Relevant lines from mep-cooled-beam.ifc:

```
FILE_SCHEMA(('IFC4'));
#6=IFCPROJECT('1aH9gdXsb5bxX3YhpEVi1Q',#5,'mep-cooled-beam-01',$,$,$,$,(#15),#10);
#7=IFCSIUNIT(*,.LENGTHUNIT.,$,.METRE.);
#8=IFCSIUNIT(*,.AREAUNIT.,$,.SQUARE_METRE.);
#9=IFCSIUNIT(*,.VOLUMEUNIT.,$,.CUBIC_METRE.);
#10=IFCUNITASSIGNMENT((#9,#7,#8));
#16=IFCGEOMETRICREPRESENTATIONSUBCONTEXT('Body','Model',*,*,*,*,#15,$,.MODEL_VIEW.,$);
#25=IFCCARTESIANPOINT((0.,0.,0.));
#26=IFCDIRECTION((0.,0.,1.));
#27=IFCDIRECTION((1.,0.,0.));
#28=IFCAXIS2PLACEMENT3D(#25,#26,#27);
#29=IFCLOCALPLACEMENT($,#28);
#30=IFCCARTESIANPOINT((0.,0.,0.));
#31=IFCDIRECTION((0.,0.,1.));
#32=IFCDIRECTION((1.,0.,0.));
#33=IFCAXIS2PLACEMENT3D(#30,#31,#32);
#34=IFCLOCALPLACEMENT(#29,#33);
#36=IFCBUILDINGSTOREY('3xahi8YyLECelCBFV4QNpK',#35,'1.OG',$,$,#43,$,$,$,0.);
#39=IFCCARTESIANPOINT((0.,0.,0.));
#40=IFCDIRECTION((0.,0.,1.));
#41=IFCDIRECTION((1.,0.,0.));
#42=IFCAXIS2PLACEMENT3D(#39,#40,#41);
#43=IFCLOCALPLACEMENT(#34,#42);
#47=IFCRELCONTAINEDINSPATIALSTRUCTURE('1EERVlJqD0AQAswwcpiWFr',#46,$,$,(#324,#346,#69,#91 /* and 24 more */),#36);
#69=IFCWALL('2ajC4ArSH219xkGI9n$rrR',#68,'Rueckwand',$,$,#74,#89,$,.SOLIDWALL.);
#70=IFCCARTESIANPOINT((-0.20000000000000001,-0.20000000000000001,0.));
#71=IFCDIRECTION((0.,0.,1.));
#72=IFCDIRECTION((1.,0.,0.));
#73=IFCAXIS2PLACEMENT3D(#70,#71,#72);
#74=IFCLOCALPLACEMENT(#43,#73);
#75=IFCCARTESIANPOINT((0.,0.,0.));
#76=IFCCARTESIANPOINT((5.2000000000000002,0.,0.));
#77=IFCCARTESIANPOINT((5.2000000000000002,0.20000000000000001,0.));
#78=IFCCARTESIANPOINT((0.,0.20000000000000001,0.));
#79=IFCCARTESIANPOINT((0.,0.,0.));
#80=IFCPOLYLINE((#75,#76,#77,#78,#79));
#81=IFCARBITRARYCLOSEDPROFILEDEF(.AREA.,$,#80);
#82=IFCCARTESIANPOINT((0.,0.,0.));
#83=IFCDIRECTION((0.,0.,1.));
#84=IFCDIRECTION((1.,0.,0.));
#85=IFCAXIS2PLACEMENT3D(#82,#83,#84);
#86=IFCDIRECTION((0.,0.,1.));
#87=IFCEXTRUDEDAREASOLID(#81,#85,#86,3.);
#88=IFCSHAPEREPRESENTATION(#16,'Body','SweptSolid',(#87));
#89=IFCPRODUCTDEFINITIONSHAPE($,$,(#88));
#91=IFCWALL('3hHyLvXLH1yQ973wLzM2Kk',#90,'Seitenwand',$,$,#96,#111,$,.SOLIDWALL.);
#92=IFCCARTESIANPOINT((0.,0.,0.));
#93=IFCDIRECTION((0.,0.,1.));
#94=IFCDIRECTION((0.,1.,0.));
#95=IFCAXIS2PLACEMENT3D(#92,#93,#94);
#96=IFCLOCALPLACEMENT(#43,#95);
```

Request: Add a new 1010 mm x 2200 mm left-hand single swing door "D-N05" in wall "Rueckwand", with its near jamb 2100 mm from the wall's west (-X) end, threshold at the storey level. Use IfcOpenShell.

```python
import numpy as np
import ifcopenshell
import ifcopenshell.api.feature
import ifcopenshell.api.geometry
import ifcopenshell.api.root
import ifcopenshell.api.spatial
import ifcopenshell.geom
import ifcopenshell.util.element
import ifcopenshell.util.placement
import ifcopenshell.util.representation
import ifcopenshell.util.shape
import ifcopenshell.util.unit

model = ifcopenshell.open("mep-cooled-beam.ifc")
unit_scale = ifcopenshell.util.unit.calculate_unit_scale(model)
settings = ifcopenshell.geom.settings()


def volume(element):
    """Net volume in cubic metres, openings subtracted."""
    shape = ifcopenshell.geom.create_shape(settings, element)
    return ifcopenshell.util.shape.get_volume(shape.geometry)


wall = model.by_guid("2ajC4ArSH219xkGI9n$rrR")
storey = ifcopenshell.util.element.get_container(wall, ifc_class="IfcBuildingStorey")
context = ifcopenshell.util.representation.get_context(model, "Model", "Body", "MODEL_VIEW")
before = volume(wall)

width, height, from_end, sill = 1.01, 2.2, 2.1, 0.0  # metres

# The wall runs along its own X axis, and the end named is its -X end.
wall_shape = ifcopenshell.geom.create_shape(settings, wall)
x, y, z = ifcopenshell.util.shape.get_vertices(wall_shape.geometry).T
start = x.min() + from_end
face, thickness = float(y.min()), float(y.max() - y.min())
wall_matrix = ifcopenshell.util.placement.get_local_placement(wall.ObjectPlacement)
level = ifcopenshell.util.placement.get_local_placement(storey.ObjectPlacement)[2, 3]


def in_wall(x, y):
    """Placement at x, y metres in the wall's axes, at sill height."""
    matrix = wall_matrix.copy()
    matrix[:, 3] = wall_matrix @ np.array([x / unit_scale, y / unit_scale, 0.0, 1.0])
    matrix[2, 3] = level + sill / unit_scale
    return matrix


# Opening: a box that overshoots both wall faces by 50 mm.
opening = ifcopenshell.api.root.create_entity(model, ifc_class="IfcOpeningElement", predefined_type="OPENING")
box = ifcopenshell.api.geometry.add_wall_representation(
    model, context=context, length=width, height=height, thickness=thickness + 0.1
)
ifcopenshell.api.geometry.assign_representation(model, product=opening, representation=box)
ifcopenshell.api.geometry.edit_object_placement(model, product=opening, matrix=in_wall(start, face - 0.05), is_si=False)
ifcopenshell.api.feature.add_feature(model, feature=opening, element=wall)

door = ifcopenshell.api.root.create_entity(model, ifc_class="IfcDoor", name="D-N05", predefined_type="DOOR")
door.OverallWidth, door.OverallHeight = width / unit_scale, height / unit_scale
door.OperationType = "SINGLE_SWING_LEFT"
body = ifcopenshell.api.geometry.add_door_representation(
    model,
    context=context,
    overall_width=door.OverallWidth,
    overall_height=door.OverallHeight,
    operation_type="SINGLE_SWING_LEFT",
    lining_properties={"LiningDepth": thickness / unit_scale, "ThresholdDepth": thickness / unit_scale},
)
ifcopenshell.api.geometry.assign_representation(model, product=door, representation=body)
ifcopenshell.api.spatial.assign_container(model, products=[door], relating_structure=storey)
ifcopenshell.api.feature.add_filling(model, opening=opening, element=door)

# The lining spans the wall, so the door starts at the wall face.
ifcopenshell.api.geometry.edit_object_placement(model, product=door, matrix=in_wall(start, face), is_si=False)

after = volume(wall)

print(f"wall volume {before:.3f} -> {after:.3f} m3")

model.write("mep-cooled-beam_rev.ifc")
```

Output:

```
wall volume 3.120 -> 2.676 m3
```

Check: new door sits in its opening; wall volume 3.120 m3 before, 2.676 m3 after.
